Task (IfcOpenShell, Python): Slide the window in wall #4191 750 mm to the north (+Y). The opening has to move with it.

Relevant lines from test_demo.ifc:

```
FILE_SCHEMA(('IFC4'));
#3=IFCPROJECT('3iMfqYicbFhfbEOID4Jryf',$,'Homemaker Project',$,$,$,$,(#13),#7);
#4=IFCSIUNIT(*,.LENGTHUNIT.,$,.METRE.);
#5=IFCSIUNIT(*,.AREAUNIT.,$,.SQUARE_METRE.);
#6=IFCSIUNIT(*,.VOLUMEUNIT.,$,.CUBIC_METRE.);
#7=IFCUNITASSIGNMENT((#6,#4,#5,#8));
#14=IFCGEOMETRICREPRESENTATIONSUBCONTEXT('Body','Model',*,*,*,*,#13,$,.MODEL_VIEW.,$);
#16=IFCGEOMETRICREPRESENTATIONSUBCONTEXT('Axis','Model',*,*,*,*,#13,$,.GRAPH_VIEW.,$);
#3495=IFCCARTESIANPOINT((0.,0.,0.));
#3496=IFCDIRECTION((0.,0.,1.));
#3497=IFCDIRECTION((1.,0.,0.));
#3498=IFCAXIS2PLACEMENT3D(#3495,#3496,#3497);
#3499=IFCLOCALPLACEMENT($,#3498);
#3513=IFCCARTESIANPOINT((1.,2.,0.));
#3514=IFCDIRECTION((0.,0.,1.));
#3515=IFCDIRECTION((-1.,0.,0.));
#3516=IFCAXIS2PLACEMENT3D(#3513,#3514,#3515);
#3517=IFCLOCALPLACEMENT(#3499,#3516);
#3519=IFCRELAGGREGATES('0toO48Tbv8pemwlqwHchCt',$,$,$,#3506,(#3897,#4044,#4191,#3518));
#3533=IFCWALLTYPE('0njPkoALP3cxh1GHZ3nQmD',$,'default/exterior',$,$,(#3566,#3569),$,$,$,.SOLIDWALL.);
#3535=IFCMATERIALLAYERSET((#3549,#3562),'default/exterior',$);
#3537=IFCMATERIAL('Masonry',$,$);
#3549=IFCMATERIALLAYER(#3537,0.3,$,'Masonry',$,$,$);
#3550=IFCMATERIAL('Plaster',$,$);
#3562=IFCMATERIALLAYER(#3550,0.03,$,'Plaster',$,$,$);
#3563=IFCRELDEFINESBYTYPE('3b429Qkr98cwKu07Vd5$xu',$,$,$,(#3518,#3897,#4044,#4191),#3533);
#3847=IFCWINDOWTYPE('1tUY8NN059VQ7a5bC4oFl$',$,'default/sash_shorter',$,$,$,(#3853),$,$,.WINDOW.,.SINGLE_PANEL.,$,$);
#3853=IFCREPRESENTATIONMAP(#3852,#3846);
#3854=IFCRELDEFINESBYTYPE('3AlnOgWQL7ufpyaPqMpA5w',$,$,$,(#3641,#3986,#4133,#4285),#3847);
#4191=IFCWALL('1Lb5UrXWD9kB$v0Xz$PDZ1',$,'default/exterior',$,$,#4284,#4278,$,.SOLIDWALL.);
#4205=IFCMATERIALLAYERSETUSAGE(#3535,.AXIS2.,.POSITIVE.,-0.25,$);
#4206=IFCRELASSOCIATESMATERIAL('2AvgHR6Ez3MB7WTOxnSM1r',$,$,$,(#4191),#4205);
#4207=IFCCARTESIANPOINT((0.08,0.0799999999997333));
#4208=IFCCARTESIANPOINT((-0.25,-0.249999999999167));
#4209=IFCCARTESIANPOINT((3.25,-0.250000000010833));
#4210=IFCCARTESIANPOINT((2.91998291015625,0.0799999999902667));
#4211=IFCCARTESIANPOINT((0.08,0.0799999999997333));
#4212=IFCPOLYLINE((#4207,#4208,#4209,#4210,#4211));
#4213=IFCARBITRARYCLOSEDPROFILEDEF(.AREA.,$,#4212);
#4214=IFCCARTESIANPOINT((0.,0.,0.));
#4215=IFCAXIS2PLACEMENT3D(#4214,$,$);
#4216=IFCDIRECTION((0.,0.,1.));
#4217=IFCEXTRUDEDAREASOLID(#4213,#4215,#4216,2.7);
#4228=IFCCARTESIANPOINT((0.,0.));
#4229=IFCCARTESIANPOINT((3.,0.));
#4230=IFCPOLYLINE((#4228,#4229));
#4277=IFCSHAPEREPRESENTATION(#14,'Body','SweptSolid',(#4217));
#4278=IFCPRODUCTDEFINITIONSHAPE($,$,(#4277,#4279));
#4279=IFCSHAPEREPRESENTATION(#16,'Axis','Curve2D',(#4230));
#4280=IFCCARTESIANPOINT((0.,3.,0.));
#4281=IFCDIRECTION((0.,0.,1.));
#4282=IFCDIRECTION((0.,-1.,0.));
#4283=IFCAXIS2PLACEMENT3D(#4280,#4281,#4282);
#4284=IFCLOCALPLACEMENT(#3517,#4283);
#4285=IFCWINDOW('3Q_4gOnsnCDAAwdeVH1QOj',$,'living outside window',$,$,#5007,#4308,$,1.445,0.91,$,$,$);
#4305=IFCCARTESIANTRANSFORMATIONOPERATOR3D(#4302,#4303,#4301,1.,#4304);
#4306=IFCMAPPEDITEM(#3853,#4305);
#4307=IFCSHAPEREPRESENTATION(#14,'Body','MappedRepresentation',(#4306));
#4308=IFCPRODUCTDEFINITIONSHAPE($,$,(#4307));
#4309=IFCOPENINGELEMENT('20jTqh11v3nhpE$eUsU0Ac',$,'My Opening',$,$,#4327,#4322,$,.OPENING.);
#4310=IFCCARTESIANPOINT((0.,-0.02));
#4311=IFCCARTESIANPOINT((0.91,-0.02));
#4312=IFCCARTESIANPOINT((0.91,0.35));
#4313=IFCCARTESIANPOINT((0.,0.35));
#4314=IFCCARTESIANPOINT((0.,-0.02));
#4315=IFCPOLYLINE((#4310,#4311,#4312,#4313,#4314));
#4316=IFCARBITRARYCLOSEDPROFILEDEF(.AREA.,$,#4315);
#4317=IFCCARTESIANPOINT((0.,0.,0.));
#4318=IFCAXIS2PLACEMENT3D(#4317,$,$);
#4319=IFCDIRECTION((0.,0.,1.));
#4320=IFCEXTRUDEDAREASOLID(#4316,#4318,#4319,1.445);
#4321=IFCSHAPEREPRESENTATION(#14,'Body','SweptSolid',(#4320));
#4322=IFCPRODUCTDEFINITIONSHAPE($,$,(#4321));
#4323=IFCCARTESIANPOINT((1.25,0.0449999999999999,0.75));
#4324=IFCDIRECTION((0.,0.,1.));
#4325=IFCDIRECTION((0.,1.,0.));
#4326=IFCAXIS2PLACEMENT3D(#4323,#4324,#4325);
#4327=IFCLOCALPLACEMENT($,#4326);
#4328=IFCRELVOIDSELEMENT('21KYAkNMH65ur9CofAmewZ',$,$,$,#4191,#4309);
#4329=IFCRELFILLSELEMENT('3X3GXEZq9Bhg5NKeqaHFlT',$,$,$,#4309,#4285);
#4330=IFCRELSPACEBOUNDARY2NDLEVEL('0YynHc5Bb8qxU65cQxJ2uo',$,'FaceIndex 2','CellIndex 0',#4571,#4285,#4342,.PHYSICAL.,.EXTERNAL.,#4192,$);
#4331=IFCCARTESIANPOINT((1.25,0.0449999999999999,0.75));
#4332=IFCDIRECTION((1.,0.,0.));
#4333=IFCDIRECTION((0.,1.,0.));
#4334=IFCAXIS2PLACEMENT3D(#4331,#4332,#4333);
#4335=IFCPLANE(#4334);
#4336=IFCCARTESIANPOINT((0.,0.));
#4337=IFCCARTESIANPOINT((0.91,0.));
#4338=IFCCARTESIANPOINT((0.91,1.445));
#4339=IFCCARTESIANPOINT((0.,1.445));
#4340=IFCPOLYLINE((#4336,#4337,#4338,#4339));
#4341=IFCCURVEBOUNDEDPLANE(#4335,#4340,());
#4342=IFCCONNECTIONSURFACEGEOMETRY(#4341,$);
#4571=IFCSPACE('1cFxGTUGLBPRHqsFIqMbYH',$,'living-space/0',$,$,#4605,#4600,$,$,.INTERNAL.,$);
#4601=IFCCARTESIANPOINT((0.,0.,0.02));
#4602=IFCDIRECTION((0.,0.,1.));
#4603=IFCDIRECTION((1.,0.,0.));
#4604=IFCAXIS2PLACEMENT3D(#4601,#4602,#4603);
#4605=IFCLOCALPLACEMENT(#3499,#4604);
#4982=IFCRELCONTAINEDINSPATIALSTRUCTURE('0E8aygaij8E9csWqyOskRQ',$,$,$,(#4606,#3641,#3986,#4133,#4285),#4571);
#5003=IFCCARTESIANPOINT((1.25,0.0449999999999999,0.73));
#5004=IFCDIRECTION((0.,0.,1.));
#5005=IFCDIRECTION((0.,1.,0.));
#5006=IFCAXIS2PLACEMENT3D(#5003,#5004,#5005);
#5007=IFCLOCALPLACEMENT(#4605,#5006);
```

```python
import numpy as np
import ifcopenshell
import ifcopenshell.api.geometry
import ifcopenshell.util.placement

model = ifcopenshell.open("test_demo.ifc")

window = model.by_id(4285)
opening = window.FillsVoids[0].RelatingOpeningElement
wall = opening.VoidsElements[0].RelatingBuildingElement

wall_matrix = ifcopenshell.util.placement.get_local_placement(wall.ObjectPlacement)
shift = wall_matrix[:3, 0] * 0.75
before = ifcopenshell.util.placement.get_local_placement(window.ObjectPlacement)[:3, 3].copy()

# The window is not placed relative to its opening, so move both.
for product in (opening, window):
    matrix = ifcopenshell.util.placement.get_local_placement(product.ObjectPlacement)
    matrix[:3, 3] += shift
    ifcopenshell.api.geometry.edit_object_placement(model, product=product, matrix=matrix, is_si=False)

# Space boundary surfaces are stored in each space's coordinates; move them too.
for rel in window.ProvidesBoundaries:
    if not rel.ConnectionGeometry:
        continue
    surface = rel.ConnectionGeometry.SurfaceOnRelatingElement.BasisSurface
    space_matrix = ifcopenshell.util.placement.get_local_placement(rel.RelatingSpace.ObjectPlacement)
    point = np.array(surface.Position.Location.Coordinates) + space_matrix[:3, :3].T @ shift
    surface.Position = model.createIfcAxis2Placement3D(
        model.createIfcCartesianPoint(point.tolist()), surface.Position.Axis, surface.Position.RefDirection
    )

after = ifcopenshell.util.placement.get_local_placement(window.ObjectPlacement)[:3, 3]
print("window moved by", (after - before).round(3) + 0.0)

model.write("test_demo-out.ifc")
```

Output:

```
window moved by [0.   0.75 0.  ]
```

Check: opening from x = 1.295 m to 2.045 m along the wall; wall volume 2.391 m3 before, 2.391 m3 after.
